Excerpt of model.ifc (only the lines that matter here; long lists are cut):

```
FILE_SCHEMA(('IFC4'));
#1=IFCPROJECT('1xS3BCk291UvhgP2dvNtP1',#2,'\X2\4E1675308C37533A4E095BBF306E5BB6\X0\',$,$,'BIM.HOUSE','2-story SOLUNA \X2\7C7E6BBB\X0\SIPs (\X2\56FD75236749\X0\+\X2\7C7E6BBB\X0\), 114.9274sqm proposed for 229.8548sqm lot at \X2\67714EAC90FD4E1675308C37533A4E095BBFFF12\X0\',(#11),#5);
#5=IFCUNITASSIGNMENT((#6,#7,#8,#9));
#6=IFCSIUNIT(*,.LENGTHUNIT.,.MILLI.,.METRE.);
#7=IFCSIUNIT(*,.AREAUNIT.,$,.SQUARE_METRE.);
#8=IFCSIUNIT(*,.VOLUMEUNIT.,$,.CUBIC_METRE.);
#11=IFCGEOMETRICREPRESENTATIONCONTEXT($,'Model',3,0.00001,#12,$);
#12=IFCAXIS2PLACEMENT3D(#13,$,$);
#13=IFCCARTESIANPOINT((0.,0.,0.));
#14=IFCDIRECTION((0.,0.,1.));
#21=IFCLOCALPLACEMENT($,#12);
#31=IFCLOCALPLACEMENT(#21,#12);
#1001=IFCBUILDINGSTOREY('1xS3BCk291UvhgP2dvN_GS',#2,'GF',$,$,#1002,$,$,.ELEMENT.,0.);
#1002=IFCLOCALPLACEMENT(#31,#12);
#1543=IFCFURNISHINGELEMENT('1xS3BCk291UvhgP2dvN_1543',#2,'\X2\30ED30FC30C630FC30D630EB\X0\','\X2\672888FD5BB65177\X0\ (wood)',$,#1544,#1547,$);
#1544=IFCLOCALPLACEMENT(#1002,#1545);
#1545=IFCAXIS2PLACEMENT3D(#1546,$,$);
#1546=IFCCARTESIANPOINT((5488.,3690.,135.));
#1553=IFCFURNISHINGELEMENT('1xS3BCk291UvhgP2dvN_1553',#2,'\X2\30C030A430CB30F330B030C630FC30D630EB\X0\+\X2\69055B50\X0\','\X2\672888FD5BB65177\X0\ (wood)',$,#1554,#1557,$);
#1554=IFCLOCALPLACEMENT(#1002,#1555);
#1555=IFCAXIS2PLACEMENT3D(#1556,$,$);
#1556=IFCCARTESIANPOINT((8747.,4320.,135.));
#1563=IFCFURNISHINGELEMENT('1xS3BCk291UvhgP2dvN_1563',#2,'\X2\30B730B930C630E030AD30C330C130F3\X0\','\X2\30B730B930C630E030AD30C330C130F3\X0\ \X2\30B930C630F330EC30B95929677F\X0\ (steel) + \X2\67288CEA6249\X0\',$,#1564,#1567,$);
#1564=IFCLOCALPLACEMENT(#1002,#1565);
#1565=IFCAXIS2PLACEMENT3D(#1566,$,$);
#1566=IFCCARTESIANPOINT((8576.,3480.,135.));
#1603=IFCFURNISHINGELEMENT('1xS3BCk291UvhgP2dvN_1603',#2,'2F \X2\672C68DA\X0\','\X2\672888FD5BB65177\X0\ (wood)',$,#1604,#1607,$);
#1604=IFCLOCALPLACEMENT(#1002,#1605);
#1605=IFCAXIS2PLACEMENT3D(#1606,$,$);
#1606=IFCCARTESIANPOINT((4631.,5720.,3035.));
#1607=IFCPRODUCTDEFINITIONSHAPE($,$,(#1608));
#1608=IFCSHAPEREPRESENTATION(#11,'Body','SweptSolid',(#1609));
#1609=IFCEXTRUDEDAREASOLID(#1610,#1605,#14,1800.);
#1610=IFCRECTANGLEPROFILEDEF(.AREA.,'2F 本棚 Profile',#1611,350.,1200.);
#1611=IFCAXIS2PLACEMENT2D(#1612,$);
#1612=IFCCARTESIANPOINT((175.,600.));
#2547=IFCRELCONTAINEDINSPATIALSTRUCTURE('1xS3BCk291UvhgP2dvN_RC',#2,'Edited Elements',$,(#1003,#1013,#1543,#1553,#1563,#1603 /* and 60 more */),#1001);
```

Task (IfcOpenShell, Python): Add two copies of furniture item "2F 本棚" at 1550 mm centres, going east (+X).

```python
import numpy as np
import ifcopenshell
import ifcopenshell.api.geometry
import ifcopenshell.api.root
import ifcopenshell.util.element
import ifcopenshell.util.placement

model = ifcopenshell.open("model.ifc")


def reuse_history(source, copy):
    """copy_class also copies each property set's owner history, people and application; keep the originals."""
    for rel in copy.IsDefinedBy:
        if rel.is_a("IfcRelDefinesByProperties") and (history := rel.RelatingPropertyDefinition.OwnerHistory):
            rel.RelatingPropertyDefinition.OwnerHistory = source.OwnerHistory
            ifcopenshell.util.element.remove_deep2(model, history)


source = model.by_id(1603)
base = ifcopenshell.util.placement.get_local_placement(source.ObjectPlacement)
step = np.array([1.0, 0.0, 0.0]) * 1550.0

for i in range(1, 3):
    copy = ifcopenshell.api.root.copy_class(model, product=source)
    copy.Representation = ifcopenshell.util.element.copy_deep(
        model, source.Representation, exclude=["IfcGeometricRepresentationContext", "IfcRepresentationMap"]
    )
    reuse_history(source, copy)
    matrix = base.copy()
    matrix[:3, 3] += i * step
    print("added at", matrix[:3, 3].round(3) + 0.0)
    ifcopenshell.api.geometry.edit_object_placement(model, product=copy, matrix=matrix, is_si=False)

model.write("model-out.ifc")
```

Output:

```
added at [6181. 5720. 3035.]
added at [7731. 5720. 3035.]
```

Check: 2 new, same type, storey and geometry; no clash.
